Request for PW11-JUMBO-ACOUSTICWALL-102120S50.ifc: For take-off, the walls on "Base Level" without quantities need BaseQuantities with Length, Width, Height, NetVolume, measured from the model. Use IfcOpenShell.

First a look at what the model holds.

```python
import ifcopenshell
import ifcopenshell.util.element
import ifcopenshell.util.unit

model = ifcopenshell.open("PW11-JUMBO-ACOUSTICWALL-102120S50.ifc")
print(model.schema)
for unit_type in ("LENGTHUNIT", "AREAUNIT", "VOLUMEUNIT"):
    print(unit_type, ifcopenshell.util.unit.calculate_unit_scale(model, unit_type))
storey = next(s for s in model.by_type("IfcBuildingStorey") if s.Name == "Base Level")
walls = [e for e in ifcopenshell.util.element.get_decomposition(storey) if e.is_a("IfcWall")]
for e in sorted(walls, key=lambda e: e.id()):
    print(e.id(), e.is_a(), e.Name, list(ifcopenshell.util.element.get_psets(e, qtos_only=True)), sep=" | ")
```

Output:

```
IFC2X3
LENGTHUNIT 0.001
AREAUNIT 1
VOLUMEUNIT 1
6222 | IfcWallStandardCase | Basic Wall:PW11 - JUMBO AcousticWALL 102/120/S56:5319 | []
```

```python
import ifcopenshell
import ifcopenshell.api.pset
import ifcopenshell.geom
import ifcopenshell.util.element
import ifcopenshell.util.shape
import ifcopenshell.util.unit

model = ifcopenshell.open("PW11-JUMBO-ACOUSTICWALL-102120S50.ifc")
unit_scale = ifcopenshell.util.unit.calculate_unit_scale(model)
volume_scale = ifcopenshell.util.unit.calculate_unit_scale(model, "VOLUMEUNIT")
settings = ifcopenshell.geom.settings()

storey = next(s for s in model.by_type("IfcBuildingStorey") if s.Name == "Base Level")
walls = [e for e in ifcopenshell.util.element.get_decomposition(storey) if e.is_a("IfcWall")]

for e in sorted(walls, key=lambda e: e.id()):
    if ifcopenshell.util.element.get_psets(e, qtos_only=True, should_inherit=False):
        continue
    # Geometry comes back in metres, in the element's own axes.
    shape = ifcopenshell.geom.create_shape(settings, e)
    values = {
        "Length": ifcopenshell.util.shape.get_x(shape.geometry) / unit_scale,
        "Width": ifcopenshell.util.shape.get_y(shape.geometry) / unit_scale,
        "Height": ifcopenshell.util.shape.get_z(shape.geometry) / unit_scale,
        "NetVolume": ifcopenshell.util.shape.get_volume(shape.geometry) / volume_scale,
    }
    qto = ifcopenshell.api.pset.add_qto(model, product=e, name="BaseQuantities")
    ifcopenshell.api.pset.edit_qto(model, qto=qto, properties=values)
    print(e.id(), {k: round(v, 3) for k, v in values.items()})

model.write("PW11-JUMBO-ACOUSTICWALL-102120S50-out.ifc")
```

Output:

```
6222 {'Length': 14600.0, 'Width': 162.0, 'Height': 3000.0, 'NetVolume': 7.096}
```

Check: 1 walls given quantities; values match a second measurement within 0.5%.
